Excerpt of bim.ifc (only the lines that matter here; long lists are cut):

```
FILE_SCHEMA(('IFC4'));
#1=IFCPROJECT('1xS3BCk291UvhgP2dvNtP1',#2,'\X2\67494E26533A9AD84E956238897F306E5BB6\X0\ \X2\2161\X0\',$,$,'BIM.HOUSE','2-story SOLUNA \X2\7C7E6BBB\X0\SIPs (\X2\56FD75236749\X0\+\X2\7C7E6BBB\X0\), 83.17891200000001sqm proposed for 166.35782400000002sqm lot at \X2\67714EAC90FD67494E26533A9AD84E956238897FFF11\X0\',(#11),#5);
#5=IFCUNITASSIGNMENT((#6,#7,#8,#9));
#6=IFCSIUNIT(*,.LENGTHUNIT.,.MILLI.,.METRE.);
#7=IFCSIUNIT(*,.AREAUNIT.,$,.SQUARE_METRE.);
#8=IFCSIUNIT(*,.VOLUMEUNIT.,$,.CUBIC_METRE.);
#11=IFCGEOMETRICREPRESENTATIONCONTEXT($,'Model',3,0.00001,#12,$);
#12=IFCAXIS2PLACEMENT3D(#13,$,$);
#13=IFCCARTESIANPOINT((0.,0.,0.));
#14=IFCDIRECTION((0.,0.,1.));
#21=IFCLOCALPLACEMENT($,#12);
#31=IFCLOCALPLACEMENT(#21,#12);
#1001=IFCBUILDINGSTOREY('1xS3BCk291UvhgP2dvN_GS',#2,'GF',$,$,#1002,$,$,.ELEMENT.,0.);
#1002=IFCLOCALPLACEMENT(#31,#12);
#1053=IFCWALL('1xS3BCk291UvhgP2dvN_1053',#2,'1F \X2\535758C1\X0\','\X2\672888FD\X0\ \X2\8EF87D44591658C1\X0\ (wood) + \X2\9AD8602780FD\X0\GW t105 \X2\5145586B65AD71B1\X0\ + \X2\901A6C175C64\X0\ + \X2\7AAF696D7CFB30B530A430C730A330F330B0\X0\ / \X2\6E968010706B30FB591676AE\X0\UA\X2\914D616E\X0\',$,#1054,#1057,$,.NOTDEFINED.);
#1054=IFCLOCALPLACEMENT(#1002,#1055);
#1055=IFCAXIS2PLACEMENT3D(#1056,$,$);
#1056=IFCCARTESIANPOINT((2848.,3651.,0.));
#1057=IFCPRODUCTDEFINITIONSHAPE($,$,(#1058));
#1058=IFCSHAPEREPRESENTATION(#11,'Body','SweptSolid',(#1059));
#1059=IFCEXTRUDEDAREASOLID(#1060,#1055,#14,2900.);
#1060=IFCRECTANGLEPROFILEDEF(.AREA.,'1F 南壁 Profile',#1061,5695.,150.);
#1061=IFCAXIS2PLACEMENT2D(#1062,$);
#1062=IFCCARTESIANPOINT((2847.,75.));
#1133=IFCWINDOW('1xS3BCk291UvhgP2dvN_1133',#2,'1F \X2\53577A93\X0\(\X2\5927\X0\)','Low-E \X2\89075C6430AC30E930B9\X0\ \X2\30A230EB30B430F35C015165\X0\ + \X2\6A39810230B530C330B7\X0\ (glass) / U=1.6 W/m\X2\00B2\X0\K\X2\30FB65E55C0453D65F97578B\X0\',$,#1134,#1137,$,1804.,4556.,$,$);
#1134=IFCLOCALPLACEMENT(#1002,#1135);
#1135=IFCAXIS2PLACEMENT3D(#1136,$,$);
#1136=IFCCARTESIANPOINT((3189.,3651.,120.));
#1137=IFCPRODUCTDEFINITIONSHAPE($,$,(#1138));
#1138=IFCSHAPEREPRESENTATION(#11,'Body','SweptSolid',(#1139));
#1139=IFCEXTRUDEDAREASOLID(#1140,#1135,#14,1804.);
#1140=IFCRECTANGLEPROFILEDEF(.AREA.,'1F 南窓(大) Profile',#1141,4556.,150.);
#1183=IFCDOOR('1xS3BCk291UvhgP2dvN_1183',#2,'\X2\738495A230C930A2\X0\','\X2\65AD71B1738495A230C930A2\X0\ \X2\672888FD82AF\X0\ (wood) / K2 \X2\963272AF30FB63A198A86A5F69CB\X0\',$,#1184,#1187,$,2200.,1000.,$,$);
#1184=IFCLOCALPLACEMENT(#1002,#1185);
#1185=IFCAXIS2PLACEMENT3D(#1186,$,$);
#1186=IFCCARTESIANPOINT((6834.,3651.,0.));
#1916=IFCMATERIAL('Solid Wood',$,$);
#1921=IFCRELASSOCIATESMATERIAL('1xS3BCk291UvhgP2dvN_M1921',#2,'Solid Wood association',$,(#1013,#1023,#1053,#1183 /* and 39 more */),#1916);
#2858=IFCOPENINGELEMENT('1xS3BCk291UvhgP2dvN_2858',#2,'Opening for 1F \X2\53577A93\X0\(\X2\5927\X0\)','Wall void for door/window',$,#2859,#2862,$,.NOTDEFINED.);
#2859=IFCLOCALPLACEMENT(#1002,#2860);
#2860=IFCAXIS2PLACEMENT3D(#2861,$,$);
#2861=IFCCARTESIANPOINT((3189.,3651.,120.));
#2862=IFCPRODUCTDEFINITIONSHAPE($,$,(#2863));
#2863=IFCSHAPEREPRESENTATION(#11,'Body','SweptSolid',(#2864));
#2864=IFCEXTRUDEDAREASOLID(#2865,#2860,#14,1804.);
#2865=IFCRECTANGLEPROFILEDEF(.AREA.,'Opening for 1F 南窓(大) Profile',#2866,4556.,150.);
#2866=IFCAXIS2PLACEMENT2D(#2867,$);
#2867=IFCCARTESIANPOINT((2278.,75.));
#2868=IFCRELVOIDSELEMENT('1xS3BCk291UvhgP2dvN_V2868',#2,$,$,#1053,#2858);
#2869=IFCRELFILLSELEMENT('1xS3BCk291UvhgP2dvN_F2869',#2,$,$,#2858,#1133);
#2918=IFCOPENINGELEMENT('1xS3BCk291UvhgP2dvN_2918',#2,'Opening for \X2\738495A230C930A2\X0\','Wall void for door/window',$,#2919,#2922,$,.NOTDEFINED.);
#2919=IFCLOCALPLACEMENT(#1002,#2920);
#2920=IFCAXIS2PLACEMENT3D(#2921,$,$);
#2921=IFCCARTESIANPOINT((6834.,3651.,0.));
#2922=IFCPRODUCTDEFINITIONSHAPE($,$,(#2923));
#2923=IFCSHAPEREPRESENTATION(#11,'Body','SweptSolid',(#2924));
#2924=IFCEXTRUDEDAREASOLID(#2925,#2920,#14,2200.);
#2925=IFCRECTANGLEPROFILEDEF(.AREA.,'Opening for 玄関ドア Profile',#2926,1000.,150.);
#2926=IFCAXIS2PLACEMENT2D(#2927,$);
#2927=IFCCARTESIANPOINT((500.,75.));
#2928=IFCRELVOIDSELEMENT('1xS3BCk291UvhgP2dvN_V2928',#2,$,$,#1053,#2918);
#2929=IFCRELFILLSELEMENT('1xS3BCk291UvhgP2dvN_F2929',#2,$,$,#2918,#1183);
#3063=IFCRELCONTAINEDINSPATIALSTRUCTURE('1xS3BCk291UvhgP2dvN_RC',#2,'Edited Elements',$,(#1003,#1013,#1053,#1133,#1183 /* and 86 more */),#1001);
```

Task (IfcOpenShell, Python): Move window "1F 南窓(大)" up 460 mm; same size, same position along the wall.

```python
import numpy as np
import ifcopenshell
import ifcopenshell.api.geometry
import ifcopenshell.util.placement
import ifcopenshell.util.unit

model = ifcopenshell.open("bim.ifc")
unit_scale = ifcopenshell.util.unit.calculate_unit_scale(model)

window = model.by_guid("1xS3BCk291UvhgP2dvN_1133")
opening = window.FillsVoids[0].RelatingOpeningElement
dz = 460.0

shift = np.array([0.0, 0.0, dz])
# The window is not placed relative to its opening, so move both.
for product in (opening, window):
    matrix = ifcopenshell.util.placement.get_local_placement(product.ObjectPlacement)
    matrix[:3, 3] += shift
    ifcopenshell.api.geometry.edit_object_placement(model, product=product, matrix=matrix, is_si=False)

print(f"moved by {dz * unit_scale:+.3f} m")

model.write("bim_v2.ifc")
```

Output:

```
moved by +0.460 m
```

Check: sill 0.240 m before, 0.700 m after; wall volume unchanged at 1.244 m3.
